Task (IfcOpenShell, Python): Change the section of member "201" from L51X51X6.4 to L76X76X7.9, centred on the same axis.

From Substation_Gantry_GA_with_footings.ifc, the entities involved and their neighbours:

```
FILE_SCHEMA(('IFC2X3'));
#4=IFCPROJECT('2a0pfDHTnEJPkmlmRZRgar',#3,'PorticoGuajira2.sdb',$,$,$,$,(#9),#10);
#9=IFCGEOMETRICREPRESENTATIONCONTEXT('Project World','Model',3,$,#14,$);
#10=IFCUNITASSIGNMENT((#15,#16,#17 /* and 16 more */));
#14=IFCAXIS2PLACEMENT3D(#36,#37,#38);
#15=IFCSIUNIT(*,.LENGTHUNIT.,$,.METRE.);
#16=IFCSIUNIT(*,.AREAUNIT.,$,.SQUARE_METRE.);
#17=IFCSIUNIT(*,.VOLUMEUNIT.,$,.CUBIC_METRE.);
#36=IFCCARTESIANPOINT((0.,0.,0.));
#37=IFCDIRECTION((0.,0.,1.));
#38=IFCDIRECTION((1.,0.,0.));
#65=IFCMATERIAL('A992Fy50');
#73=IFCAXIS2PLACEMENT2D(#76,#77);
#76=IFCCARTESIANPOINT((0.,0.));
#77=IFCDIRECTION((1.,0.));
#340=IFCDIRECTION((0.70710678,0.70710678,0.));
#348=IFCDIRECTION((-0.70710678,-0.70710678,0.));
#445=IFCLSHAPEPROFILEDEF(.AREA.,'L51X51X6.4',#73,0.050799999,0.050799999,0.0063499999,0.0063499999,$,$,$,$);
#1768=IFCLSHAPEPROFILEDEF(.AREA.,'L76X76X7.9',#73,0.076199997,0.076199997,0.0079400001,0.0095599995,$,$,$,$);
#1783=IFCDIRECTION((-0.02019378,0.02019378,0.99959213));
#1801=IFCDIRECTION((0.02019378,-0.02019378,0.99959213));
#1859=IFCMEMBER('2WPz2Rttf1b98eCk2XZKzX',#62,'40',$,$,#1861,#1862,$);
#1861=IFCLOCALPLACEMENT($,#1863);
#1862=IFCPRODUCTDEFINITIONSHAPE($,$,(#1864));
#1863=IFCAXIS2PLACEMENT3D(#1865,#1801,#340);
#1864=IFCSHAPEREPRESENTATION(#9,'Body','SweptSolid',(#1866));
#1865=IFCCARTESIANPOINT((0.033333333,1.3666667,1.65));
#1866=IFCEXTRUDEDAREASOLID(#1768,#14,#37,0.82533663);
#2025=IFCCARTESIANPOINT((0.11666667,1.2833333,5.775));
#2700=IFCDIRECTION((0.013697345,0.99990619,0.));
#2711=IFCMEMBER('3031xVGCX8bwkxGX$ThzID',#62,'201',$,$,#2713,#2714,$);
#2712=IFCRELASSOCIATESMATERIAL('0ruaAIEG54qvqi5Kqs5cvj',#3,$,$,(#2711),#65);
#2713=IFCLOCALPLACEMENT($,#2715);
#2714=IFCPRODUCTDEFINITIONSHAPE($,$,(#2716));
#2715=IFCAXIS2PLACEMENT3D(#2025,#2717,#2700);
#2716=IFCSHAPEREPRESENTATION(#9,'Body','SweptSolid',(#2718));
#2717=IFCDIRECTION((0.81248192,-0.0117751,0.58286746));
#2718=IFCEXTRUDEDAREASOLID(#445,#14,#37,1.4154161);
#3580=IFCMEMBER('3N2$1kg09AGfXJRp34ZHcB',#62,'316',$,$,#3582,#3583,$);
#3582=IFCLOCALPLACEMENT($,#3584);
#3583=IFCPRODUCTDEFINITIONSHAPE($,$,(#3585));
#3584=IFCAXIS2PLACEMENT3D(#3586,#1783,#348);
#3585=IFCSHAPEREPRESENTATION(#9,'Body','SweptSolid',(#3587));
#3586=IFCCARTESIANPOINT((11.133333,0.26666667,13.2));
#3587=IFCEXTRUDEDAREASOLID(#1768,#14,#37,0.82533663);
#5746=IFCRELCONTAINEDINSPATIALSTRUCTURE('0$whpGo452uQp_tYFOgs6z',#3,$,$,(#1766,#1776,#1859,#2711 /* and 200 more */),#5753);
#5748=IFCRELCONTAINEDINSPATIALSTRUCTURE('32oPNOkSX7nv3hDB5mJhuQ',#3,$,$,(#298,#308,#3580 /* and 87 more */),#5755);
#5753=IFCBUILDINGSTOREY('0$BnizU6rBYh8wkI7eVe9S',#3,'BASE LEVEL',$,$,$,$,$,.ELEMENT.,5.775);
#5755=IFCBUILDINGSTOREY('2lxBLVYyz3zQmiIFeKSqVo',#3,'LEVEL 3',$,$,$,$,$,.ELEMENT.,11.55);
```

```python
import ifcopenshell
import ifcopenshell.util.element

model = ifcopenshell.open("Substation_Gantry_GA_with_footings.ifc")

member = model.by_guid("3031xVGCX8bwkxGX$ThzID")
source = next(p for p in model.by_type("IfcLShapeProfileDef") if p.ProfileName == "L76X76X7.9")

body = next(r for r in member.Representation.Representations if r.RepresentationIdentifier == "Body")
solid = body.Items[0]
old_profile = solid.SweptArea

# Copy the section's sizes but keep this member's own profile position.
profile = ifcopenshell.util.element.copy(model, source)
profile.Position = old_profile.Position
solid.SweptArea = profile
if not model.get_total_inverses(old_profile):
    ifcopenshell.util.element.remove_deep2(model, old_profile)

print(solid.SweptArea)

model.write("Substation_Gantry_GA_with_footings-out.ifc")
```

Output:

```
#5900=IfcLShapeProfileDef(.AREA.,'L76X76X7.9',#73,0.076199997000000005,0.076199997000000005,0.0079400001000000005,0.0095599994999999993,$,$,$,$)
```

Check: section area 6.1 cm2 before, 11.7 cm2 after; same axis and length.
